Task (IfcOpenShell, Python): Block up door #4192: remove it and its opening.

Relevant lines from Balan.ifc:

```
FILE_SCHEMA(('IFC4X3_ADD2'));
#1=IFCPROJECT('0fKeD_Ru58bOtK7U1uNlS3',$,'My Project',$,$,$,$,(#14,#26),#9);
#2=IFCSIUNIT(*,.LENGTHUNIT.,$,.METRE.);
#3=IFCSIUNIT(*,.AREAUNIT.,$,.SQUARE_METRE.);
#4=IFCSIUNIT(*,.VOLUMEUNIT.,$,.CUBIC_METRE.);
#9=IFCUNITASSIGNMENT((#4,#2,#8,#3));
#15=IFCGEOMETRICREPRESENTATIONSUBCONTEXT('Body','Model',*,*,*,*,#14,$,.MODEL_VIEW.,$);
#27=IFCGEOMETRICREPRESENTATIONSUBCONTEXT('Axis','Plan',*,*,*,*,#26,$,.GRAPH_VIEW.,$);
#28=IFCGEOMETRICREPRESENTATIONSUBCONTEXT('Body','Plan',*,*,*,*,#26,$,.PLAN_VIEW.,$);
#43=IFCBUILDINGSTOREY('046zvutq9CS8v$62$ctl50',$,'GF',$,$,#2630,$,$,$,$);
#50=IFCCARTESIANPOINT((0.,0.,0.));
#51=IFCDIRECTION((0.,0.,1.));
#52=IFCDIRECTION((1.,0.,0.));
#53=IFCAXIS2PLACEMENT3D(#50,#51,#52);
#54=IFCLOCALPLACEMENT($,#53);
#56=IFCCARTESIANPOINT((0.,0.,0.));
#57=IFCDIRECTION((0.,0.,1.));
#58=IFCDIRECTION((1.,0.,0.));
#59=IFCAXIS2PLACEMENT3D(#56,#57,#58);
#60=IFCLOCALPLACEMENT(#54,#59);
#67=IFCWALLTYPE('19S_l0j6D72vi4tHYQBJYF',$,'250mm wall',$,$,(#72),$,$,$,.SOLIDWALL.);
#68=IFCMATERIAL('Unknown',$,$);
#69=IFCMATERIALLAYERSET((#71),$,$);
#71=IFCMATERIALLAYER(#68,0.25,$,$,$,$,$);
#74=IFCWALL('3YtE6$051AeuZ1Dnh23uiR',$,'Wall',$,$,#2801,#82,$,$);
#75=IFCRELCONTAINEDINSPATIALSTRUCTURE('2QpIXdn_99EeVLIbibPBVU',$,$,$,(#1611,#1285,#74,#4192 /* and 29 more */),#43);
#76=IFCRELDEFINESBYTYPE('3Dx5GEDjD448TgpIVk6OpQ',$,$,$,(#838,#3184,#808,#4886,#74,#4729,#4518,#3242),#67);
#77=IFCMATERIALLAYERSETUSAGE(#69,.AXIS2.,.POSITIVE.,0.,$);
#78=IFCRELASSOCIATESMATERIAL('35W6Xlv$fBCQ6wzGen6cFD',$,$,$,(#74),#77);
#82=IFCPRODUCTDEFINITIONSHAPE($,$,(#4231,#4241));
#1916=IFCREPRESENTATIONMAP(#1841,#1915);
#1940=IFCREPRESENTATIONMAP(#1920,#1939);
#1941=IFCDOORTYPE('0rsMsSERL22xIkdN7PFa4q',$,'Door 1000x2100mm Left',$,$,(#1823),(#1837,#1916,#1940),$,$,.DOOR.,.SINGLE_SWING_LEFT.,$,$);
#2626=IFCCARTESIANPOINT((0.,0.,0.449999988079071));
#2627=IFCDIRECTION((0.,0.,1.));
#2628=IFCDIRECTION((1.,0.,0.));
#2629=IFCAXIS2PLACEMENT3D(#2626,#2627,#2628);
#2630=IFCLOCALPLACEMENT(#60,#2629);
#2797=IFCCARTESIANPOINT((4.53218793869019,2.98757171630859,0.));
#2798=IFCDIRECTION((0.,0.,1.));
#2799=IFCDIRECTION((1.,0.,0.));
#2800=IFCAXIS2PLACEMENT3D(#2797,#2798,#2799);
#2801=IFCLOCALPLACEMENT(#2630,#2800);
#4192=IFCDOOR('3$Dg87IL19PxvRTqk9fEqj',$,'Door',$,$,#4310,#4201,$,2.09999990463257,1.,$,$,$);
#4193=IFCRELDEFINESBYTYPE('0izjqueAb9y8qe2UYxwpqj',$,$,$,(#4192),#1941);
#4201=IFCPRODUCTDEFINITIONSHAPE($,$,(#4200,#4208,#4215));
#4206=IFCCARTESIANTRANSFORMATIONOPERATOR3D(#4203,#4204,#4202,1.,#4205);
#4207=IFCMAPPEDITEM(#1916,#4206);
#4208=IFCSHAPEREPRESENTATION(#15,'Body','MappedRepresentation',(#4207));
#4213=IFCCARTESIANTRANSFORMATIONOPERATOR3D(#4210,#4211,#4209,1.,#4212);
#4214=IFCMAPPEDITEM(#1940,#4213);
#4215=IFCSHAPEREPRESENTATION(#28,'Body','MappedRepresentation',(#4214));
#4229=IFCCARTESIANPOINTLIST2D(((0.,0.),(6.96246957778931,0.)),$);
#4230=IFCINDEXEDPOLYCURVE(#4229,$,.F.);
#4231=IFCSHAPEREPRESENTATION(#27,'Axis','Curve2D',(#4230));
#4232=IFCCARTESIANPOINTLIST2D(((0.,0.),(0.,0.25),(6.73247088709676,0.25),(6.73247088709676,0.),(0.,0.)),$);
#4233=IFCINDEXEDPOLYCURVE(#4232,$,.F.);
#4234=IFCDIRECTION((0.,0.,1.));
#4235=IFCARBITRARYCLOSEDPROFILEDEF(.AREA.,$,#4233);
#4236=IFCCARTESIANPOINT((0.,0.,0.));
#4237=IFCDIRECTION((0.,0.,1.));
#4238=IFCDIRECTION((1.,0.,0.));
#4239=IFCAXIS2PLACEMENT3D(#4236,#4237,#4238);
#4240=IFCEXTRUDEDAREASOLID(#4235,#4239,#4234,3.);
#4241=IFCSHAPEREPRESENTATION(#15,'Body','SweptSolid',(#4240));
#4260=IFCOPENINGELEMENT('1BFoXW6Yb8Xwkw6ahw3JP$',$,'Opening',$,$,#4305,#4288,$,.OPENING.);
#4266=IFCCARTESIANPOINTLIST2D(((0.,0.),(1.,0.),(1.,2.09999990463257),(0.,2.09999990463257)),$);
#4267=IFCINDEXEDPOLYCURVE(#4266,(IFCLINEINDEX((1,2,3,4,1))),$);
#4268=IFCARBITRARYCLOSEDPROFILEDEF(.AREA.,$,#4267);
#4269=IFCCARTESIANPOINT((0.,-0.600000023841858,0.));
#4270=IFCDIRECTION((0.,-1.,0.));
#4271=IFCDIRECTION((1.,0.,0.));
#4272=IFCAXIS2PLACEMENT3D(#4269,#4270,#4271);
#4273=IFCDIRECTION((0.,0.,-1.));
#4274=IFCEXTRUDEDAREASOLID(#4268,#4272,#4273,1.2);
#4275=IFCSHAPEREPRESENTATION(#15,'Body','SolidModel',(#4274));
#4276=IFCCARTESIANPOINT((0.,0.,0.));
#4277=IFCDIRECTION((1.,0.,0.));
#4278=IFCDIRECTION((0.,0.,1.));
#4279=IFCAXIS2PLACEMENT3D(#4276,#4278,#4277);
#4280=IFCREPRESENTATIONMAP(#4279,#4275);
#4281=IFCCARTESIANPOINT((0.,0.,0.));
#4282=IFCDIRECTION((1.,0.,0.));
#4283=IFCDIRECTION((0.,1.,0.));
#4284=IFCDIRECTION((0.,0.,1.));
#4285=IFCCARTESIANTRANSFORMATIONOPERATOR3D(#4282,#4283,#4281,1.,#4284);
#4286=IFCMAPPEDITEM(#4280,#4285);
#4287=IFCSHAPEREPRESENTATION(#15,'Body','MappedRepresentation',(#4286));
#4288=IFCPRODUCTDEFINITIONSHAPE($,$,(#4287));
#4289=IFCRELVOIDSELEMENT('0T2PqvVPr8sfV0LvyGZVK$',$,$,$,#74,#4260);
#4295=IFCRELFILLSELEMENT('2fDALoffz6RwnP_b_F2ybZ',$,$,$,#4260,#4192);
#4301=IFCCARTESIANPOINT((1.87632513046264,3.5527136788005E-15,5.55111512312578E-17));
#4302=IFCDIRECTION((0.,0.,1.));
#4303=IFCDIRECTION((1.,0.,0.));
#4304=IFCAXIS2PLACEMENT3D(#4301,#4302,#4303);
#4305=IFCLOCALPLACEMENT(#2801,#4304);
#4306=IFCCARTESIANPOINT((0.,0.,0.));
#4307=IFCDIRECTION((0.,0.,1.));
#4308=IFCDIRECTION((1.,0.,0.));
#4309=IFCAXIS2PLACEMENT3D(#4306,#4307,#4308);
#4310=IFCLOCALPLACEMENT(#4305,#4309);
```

```python
import ifcopenshell
import ifcopenshell.api.feature
import ifcopenshell.api.root
import ifcopenshell.geom
import ifcopenshell.util.shape

model = ifcopenshell.open("Balan.ifc")
settings = ifcopenshell.geom.settings()


def volume(element):
    """Net volume in cubic metres, openings subtracted."""
    shape = ifcopenshell.geom.create_shape(settings, element)
    return ifcopenshell.util.shape.get_volume(shape.geometry)


door = model.by_guid("3$Dg87IL19PxvRTqk9fEqj")
opening = door.FillsVoids[0].RelatingOpeningElement
wall = opening.VoidsElements[0].RelatingBuildingElement
before = volume(wall)

ifcopenshell.api.root.remove_product(model, product=door)
ifcopenshell.api.feature.remove_feature(model, feature=opening)

after = volume(wall)

print(f"wall volume {before:.3f} -> {after:.3f} m3")

model.write("Balan_edited.ifc")
```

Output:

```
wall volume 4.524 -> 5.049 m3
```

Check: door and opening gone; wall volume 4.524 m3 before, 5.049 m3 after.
